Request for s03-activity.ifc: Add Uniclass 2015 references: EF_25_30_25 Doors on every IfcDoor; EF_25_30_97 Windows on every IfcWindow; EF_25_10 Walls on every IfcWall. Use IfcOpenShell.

First a look at what the model holds.

```python
import ifcopenshell

model = ifcopenshell.open("s03-activity.ifc")
print(model.schema)
print("classifications:", [c.Name for c in model.by_type("IfcClassification")])
for ifc_class in ("IfcDoor", "IfcRoof", "IfcStair", "IfcWall", "IfcWindow"):
    print(ifc_class, len(model.by_type(ifc_class)))
```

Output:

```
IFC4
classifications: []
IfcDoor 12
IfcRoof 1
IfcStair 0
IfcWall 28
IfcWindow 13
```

```python
import ifcopenshell
import ifcopenshell.api.classification

model = ifcopenshell.open("s03-activity.ifc")

system = ifcopenshell.api.classification.add_classification(model, classification="Uniclass 2015")

codes = {
    "IfcDoor": ("EF_25_30_25", "Doors"),
    "IfcWindow": ("EF_25_30_97", "Windows"),
    "IfcWall": ("EF_25_10", "Walls"),
}
for ifc_class, (code, name) in codes.items():
    products = model.by_type(ifc_class)
    ifcopenshell.api.classification.add_reference(
        model, products=products, classification=system, identification=code, name=name
    )
    print(code, len(products))

model.write("s03-activity_v2.ifc")
```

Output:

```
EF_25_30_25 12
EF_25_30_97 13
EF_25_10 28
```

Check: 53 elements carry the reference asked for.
